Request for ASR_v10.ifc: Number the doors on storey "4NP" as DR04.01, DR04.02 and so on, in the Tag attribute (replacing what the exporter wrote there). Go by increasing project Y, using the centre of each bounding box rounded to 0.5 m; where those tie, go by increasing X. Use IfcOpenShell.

First a look at what the model holds.

```python
import ifcopenshell
import ifcopenshell.util.element
import ifcopenshell.util.placement

model = ifcopenshell.open("ASR_v10.ifc")
print(model.schema)
storey = next(s for s in model.by_type("IfcBuildingStorey") if s.Name == "4NP")
doors = [e for e in ifcopenshell.util.element.get_decomposition(storey) if e.is_a("IfcDoor")]
for e in sorted(doors, key=lambda e: e.id()):
    origin = ifcopenshell.util.placement.get_local_placement(e.ObjectPlacement)[:3, 3]
    print(e.id(), e.Tag, e.Name, origin.round(2) + 0.0, sep=" | ")
```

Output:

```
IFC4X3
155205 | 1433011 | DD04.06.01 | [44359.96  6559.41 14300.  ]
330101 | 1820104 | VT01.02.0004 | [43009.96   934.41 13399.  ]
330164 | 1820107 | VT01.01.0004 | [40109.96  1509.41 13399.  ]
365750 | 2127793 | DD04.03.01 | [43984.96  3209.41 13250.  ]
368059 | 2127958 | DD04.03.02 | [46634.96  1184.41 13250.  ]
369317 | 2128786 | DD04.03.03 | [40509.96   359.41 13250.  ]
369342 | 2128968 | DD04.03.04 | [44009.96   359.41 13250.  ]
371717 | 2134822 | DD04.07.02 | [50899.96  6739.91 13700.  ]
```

```python
import ifcopenshell
import ifcopenshell.geom
import ifcopenshell.util.element
import ifcopenshell.util.shape

model = ifcopenshell.open("ASR_v10.ifc")
settings = ifcopenshell.geom.settings()
settings.set("use-world-coords", True)


def centre(element):
    shape = ifcopenshell.geom.create_shape(settings, element)
    return ifcopenshell.util.shape.get_bbox_centroid(shape.geometry)


storey = next(s for s in model.by_type("IfcBuildingStorey") if s.Name == "4NP")
doors = [e for e in ifcopenshell.util.element.get_decomposition(storey) if e.is_a("IfcDoor")]

# Insertion points can sit at a corner or the storey origin, so sort by the geometry (in metres).
centres = {e: centre(e) for e in doors}
doors.sort(key=lambda e: (round(centres[e][1] / 0.5), centres[e][0]))

for i, e in enumerate(doors, start=1):
    number = f"DR04.{i:02d}"
    e.Tag = number
    print(e.id(), number)

model.write("ASR_v10_updated.ifc")
```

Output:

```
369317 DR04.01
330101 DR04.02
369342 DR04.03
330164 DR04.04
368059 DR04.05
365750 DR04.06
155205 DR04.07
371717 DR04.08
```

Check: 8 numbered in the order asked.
